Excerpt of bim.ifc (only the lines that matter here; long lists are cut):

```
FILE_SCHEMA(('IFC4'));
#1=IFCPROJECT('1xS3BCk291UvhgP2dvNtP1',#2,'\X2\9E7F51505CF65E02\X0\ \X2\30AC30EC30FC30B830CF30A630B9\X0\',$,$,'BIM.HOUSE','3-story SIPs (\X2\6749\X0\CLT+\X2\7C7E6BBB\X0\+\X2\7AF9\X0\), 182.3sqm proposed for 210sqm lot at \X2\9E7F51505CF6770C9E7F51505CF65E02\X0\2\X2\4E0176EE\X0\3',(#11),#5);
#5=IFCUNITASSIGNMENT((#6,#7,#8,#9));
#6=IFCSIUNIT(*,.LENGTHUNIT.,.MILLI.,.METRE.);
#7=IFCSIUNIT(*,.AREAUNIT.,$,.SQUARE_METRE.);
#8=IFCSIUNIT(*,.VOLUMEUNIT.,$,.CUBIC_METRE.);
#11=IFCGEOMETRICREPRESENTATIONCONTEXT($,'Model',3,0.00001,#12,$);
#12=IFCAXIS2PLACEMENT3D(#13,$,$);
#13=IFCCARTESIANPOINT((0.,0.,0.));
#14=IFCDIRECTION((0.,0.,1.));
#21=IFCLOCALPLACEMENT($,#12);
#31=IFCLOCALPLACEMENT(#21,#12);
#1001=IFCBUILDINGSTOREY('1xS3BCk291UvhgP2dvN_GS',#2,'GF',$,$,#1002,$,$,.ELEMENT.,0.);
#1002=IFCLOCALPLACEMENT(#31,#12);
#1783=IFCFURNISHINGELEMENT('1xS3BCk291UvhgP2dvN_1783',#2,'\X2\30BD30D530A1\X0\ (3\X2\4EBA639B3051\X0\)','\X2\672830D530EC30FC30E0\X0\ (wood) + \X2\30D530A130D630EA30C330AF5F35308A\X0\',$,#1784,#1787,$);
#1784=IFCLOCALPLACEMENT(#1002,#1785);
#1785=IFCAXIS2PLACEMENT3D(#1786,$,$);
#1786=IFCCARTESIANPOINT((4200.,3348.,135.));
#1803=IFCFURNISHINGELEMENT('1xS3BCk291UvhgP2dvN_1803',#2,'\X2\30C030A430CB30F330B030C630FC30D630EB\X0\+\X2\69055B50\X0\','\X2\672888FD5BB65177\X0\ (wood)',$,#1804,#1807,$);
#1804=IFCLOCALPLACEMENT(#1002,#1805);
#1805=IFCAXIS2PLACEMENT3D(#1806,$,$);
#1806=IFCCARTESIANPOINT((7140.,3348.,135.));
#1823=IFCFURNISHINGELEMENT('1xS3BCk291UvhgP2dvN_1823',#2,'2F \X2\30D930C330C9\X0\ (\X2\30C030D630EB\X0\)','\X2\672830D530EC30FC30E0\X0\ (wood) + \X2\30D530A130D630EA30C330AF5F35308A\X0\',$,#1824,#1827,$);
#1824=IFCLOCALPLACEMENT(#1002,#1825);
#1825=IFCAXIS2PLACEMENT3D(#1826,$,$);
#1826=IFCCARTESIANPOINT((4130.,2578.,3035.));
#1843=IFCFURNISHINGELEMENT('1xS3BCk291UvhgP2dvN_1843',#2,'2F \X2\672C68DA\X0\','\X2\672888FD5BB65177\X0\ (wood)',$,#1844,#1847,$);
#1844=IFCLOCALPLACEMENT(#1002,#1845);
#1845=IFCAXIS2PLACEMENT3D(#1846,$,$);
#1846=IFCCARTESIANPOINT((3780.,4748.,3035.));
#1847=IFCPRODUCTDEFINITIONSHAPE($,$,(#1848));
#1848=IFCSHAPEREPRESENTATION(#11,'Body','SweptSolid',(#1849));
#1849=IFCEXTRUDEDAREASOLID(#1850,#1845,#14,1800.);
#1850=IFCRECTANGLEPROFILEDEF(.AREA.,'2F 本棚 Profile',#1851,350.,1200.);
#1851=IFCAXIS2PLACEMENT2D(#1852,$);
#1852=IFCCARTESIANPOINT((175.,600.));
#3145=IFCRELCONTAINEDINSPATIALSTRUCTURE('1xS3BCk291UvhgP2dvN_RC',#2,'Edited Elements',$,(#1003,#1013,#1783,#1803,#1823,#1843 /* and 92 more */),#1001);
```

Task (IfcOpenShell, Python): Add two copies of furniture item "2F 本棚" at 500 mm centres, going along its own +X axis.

```python
import ifcopenshell
import ifcopenshell.api.geometry
import ifcopenshell.api.root
import ifcopenshell.util.element
import ifcopenshell.util.placement
import ifcopenshell.util.unit

model = ifcopenshell.open("bim.ifc")
unit_scale = ifcopenshell.util.unit.calculate_unit_scale(model)


def reuse_history(source, copy):
    """copy_class also copies each property set's owner history, people and application; keep the originals."""
    for rel in copy.IsDefinedBy:
        if rel.is_a("IfcRelDefinesByProperties") and (history := rel.RelatingPropertyDefinition.OwnerHistory):
            rel.RelatingPropertyDefinition.OwnerHistory = source.OwnerHistory
            ifcopenshell.util.element.remove_deep2(model, history)


source = model.by_guid("1xS3BCk291UvhgP2dvN_1843")
base = ifcopenshell.util.placement.get_local_placement(source.ObjectPlacement)
step = base[:3, 0] * 0.5 / unit_scale

for i in range(1, 3):
    copy = ifcopenshell.api.root.copy_class(model, product=source)
    copy.Representation = ifcopenshell.util.element.copy_deep(
        model, source.Representation, exclude=["IfcGeometricRepresentationContext", "IfcRepresentationMap"]
    )
    reuse_history(source, copy)
    matrix = base.copy()
    matrix[:3, 3] += i * step
    print("added at", matrix[:3, 3].round(3) + 0.0)
    ifcopenshell.api.geometry.edit_object_placement(model, product=copy, matrix=matrix, is_si=False)

model.write("bim_v2.ifc")
```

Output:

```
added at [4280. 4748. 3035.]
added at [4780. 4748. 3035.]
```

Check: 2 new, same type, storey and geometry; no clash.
